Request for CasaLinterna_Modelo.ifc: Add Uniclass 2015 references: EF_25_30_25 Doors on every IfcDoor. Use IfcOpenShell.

First a look at what the model holds.

```python
import ifcopenshell

model = ifcopenshell.open("CasaLinterna_Modelo.ifc")
print(model.schema)
print("classifications:", [c.Name for c in model.by_type("IfcClassification")])
for ifc_class in ("IfcDoor", "IfcRoof", "IfcStair", "IfcWall", "IfcWindow"):
    print(ifc_class, len(model.by_type(ifc_class)))
```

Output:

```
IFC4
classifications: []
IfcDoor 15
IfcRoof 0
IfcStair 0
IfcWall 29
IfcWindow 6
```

```python
import ifcopenshell
import ifcopenshell.api.classification

model = ifcopenshell.open("CasaLinterna_Modelo.ifc")

system = ifcopenshell.api.classification.add_classification(model, classification="Uniclass 2015")

codes = {
    "IfcDoor": ("EF_25_30_25", "Doors"),
}
for ifc_class, (code, name) in codes.items():
    products = model.by_type(ifc_class)
    ifcopenshell.api.classification.add_reference(
        model, products=products, classification=system, identification=code, name=name
    )
    print(code, len(products))

model.write("CasaLinterna_Modelo_edited.ifc")
```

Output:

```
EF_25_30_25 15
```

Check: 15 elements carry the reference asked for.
